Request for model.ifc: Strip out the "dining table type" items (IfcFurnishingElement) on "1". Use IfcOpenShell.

First a look at what the model holds.

```python
import ifcopenshell
import ifcopenshell.util.element

model = ifcopenshell.open("model.ifc")
print(model.schema)
storey = next(s for s in model.by_type("IfcBuildingStorey") if s.Name == "1")
furniture = [e for e in ifcopenshell.util.element.get_decomposition(storey) if e.is_a("IfcFurnishingElement")]
seen = {}
for e in furniture:
    element_type = ifcopenshell.util.element.get_type(e)
    name = element_type.Name if element_type not in (None, e) else None
    seen[name] = seen.get(name, 0) + 1
for name, count in sorted(seen.items(), key=str):
    print(count, "x", name)
```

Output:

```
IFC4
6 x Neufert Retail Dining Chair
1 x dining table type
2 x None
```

```python
import ifcopenshell
import ifcopenshell.api.root
import ifcopenshell.util.element

model = ifcopenshell.open("model.ifc")

storey = next(s for s in model.by_type("IfcBuildingStorey") if s.Name == "1")
furniture = [e for e in ifcopenshell.util.element.get_decomposition(storey) if e.is_a("IfcFurnishingElement")]
targets = [e for e in furniture if (t := ifcopenshell.util.element.get_type(e)) not in (None, e) and t.Name == "dining table type"]

for e in targets:
    ifcopenshell.api.root.remove_product(model, product=e)
print(len(targets), "removed")

model.write("model-out.ifc")
```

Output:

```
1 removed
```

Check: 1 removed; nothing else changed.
